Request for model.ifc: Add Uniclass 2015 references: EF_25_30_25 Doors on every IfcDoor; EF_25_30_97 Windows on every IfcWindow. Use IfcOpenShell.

First a look at what the model holds.

```python
import ifcopenshell

model = ifcopenshell.open("model.ifc")
print(model.schema)
print("classifications:", [c.Name for c in model.by_type("IfcClassification")])
for ifc_class in ("IfcDoor", "IfcRoof", "IfcStair", "IfcWall", "IfcWindow"):
    print(ifc_class, len(model.by_type(ifc_class)))
```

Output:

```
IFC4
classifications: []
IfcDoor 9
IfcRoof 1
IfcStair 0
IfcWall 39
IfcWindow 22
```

```python
import ifcopenshell
import ifcopenshell.api.classification

model = ifcopenshell.open("model.ifc")

system = ifcopenshell.api.classification.add_classification(model, classification="Uniclass 2015")

codes = {
    "IfcDoor": ("EF_25_30_25", "Doors"),
    "IfcWindow": ("EF_25_30_97", "Windows"),
}
for ifc_class, (code, name) in codes.items():
    products = model.by_type(ifc_class)
    ifcopenshell.api.classification.add_reference(
        model, products=products, classification=system, identification=code, name=name
    )
    print(code, len(products))

model.write("model_edited.ifc")
```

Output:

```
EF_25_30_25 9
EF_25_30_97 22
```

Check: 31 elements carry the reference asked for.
